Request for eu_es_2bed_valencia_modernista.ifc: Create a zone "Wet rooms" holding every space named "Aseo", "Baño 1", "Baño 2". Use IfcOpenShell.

First a look at what the model holds.

```python
import ifcopenshell

model = ifcopenshell.open("eu_es_2bed_valencia_modernista.ifc")
print(model.schema)
seen = {}
for space in model.by_type("IfcSpace"):
    seen[space.LongName] = seen.get(space.LongName, 0) + 1
for name, count in sorted(seen.items(), key=str):
    print(count, "x", name)
print("zones:", [z.Name for z in model.by_type("IfcZone")][:20])
```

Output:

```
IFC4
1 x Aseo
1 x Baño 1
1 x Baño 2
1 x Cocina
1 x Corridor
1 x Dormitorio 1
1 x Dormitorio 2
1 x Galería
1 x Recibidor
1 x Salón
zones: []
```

```python
import ifcopenshell
import ifcopenshell.api.group
import ifcopenshell.api.root

model = ifcopenshell.open("eu_es_2bed_valencia_modernista.ifc")

names = {"Aseo", "Baño 1", "Baño 2"}
spaces = [s for s in model.by_type("IfcSpace") if s.LongName in names]

zone = ifcopenshell.api.root.create_entity(model, ifc_class="IfcZone", name="Wet rooms")
ifcopenshell.api.group.assign_group(model, products=spaces, group=zone)
print(len(spaces), "spaces in", zone.Name)

model.write("eu_es_2bed_valencia_modernista-out.ifc")
```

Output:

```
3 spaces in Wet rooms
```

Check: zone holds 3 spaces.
